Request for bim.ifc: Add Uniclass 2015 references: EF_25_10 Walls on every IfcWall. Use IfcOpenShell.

First a look at what the model holds.

```python
import ifcopenshell

model = ifcopenshell.open("bim.ifc")
print(model.schema)
print("classifications:", [c.Name for c in model.by_type("IfcClassification")])
for ifc_class in ("IfcDoor", "IfcRoof", "IfcStair", "IfcWall", "IfcWindow"):
    print(ifc_class, len(model.by_type(ifc_class)))
```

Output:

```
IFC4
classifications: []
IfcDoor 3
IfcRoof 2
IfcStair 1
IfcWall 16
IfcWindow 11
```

```python
import ifcopenshell
import ifcopenshell.api.classification

model = ifcopenshell.open("bim.ifc")

system = ifcopenshell.api.classification.add_classification(model, classification="Uniclass 2015")

codes = {
    "IfcWall": ("EF_25_10", "Walls"),
}
for ifc_class, (code, name) in codes.items():
    products = model.by_type(ifc_class)
    ifcopenshell.api.classification.add_reference(
        model, products=products, classification=system, identification=code, name=name
    )
    print(code, len(products))

model.write("bim_edited.ifc")
```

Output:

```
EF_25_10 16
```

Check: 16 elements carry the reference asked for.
